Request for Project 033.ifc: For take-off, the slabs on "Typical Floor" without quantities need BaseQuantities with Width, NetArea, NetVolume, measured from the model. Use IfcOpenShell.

First a look at what the model holds.

```python
import ifcopenshell
import ifcopenshell.util.element
import ifcopenshell.util.unit

model = ifcopenshell.open("Project 033.ifc")
print(model.schema)
for unit_type in ("LENGTHUNIT", "AREAUNIT", "VOLUMEUNIT"):
    print(unit_type, ifcopenshell.util.unit.calculate_unit_scale(model, unit_type))
storey = next(s for s in model.by_type("IfcBuildingStorey") if s.Name == "Typical Floor")
slabs = [e for e in ifcopenshell.util.element.get_decomposition(storey) if e.is_a("IfcSlab")]
for e in sorted(slabs, key=lambda e: e.id()):
    print(e.id(), e.is_a(), e.Name, list(ifcopenshell.util.element.get_psets(e, qtos_only=True)), sep=" | ")
```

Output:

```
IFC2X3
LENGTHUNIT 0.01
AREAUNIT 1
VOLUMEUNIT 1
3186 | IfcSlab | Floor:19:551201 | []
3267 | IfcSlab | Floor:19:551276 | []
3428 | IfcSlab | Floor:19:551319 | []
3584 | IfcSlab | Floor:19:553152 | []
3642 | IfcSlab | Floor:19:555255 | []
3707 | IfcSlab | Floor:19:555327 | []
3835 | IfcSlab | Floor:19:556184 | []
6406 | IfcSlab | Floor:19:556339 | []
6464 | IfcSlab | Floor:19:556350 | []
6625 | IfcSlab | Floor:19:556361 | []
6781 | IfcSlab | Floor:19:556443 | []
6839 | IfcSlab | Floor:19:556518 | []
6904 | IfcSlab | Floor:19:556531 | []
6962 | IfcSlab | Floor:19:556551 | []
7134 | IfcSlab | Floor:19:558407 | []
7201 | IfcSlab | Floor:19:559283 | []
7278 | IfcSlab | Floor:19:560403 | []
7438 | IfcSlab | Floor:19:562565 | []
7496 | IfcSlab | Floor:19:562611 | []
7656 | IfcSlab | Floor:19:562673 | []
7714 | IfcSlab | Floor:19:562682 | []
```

```python
import ifcopenshell
import ifcopenshell.api.pset
import ifcopenshell.geom
import ifcopenshell.util.element
import ifcopenshell.util.shape
import ifcopenshell.util.unit

model = ifcopenshell.open("Project 033.ifc")
unit_scale = ifcopenshell.util.unit.calculate_unit_scale(model)
area_scale = ifcopenshell.util.unit.calculate_unit_scale(model, "AREAUNIT")
volume_scale = ifcopenshell.util.unit.calculate_unit_scale(model, "VOLUMEUNIT")
settings = ifcopenshell.geom.settings()

storey = next(s for s in model.by_type("IfcBuildingStorey") if s.Name == "Typical Floor")
slabs = [e for e in ifcopenshell.util.element.get_decomposition(storey) if e.is_a("IfcSlab")]

for e in sorted(slabs, key=lambda e: e.id()):
    if ifcopenshell.util.element.get_psets(e, qtos_only=True, should_inherit=False):
        continue
    # Geometry comes back in metres, in the element's own axes.
    shape = ifcopenshell.geom.create_shape(settings, e)
    values = {
        "Width": ifcopenshell.util.shape.get_z(shape.geometry) / unit_scale,
        "NetArea": ifcopenshell.util.shape.get_footprint_area(shape.geometry) / area_scale,
        "NetVolume": ifcopenshell.util.shape.get_volume(shape.geometry) / volume_scale,
    }
    qto = ifcopenshell.api.pset.add_qto(model, product=e, name="BaseQuantities")
    ifcopenshell.api.pset.edit_qto(model, qto=qto, properties=values)
    print(e.id(), {k: round(v, 3) for k, v in values.items()})

model.write("Project 033-out.ifc")
```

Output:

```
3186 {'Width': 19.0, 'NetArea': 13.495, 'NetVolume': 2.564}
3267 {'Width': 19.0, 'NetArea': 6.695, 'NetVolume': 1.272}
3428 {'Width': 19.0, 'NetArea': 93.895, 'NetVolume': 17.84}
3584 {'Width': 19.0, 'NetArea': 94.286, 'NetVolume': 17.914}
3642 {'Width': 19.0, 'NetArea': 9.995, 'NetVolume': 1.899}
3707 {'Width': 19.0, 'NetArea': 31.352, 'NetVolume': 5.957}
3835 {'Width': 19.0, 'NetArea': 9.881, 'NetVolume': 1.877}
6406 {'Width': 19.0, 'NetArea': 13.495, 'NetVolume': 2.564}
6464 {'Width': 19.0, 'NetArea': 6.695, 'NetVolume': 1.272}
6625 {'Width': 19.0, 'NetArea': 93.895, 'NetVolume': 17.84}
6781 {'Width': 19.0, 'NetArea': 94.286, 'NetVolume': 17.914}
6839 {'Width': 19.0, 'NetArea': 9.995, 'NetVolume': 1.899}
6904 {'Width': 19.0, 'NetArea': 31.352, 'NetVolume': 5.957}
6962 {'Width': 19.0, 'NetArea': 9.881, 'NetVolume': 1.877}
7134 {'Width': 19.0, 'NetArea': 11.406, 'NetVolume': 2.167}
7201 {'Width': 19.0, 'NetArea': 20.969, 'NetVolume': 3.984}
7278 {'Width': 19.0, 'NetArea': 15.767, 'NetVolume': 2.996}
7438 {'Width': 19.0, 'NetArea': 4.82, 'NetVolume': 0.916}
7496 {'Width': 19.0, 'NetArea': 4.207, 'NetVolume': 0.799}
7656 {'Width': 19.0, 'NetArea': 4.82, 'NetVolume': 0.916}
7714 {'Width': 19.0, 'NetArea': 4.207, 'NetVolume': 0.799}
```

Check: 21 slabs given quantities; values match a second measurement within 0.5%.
